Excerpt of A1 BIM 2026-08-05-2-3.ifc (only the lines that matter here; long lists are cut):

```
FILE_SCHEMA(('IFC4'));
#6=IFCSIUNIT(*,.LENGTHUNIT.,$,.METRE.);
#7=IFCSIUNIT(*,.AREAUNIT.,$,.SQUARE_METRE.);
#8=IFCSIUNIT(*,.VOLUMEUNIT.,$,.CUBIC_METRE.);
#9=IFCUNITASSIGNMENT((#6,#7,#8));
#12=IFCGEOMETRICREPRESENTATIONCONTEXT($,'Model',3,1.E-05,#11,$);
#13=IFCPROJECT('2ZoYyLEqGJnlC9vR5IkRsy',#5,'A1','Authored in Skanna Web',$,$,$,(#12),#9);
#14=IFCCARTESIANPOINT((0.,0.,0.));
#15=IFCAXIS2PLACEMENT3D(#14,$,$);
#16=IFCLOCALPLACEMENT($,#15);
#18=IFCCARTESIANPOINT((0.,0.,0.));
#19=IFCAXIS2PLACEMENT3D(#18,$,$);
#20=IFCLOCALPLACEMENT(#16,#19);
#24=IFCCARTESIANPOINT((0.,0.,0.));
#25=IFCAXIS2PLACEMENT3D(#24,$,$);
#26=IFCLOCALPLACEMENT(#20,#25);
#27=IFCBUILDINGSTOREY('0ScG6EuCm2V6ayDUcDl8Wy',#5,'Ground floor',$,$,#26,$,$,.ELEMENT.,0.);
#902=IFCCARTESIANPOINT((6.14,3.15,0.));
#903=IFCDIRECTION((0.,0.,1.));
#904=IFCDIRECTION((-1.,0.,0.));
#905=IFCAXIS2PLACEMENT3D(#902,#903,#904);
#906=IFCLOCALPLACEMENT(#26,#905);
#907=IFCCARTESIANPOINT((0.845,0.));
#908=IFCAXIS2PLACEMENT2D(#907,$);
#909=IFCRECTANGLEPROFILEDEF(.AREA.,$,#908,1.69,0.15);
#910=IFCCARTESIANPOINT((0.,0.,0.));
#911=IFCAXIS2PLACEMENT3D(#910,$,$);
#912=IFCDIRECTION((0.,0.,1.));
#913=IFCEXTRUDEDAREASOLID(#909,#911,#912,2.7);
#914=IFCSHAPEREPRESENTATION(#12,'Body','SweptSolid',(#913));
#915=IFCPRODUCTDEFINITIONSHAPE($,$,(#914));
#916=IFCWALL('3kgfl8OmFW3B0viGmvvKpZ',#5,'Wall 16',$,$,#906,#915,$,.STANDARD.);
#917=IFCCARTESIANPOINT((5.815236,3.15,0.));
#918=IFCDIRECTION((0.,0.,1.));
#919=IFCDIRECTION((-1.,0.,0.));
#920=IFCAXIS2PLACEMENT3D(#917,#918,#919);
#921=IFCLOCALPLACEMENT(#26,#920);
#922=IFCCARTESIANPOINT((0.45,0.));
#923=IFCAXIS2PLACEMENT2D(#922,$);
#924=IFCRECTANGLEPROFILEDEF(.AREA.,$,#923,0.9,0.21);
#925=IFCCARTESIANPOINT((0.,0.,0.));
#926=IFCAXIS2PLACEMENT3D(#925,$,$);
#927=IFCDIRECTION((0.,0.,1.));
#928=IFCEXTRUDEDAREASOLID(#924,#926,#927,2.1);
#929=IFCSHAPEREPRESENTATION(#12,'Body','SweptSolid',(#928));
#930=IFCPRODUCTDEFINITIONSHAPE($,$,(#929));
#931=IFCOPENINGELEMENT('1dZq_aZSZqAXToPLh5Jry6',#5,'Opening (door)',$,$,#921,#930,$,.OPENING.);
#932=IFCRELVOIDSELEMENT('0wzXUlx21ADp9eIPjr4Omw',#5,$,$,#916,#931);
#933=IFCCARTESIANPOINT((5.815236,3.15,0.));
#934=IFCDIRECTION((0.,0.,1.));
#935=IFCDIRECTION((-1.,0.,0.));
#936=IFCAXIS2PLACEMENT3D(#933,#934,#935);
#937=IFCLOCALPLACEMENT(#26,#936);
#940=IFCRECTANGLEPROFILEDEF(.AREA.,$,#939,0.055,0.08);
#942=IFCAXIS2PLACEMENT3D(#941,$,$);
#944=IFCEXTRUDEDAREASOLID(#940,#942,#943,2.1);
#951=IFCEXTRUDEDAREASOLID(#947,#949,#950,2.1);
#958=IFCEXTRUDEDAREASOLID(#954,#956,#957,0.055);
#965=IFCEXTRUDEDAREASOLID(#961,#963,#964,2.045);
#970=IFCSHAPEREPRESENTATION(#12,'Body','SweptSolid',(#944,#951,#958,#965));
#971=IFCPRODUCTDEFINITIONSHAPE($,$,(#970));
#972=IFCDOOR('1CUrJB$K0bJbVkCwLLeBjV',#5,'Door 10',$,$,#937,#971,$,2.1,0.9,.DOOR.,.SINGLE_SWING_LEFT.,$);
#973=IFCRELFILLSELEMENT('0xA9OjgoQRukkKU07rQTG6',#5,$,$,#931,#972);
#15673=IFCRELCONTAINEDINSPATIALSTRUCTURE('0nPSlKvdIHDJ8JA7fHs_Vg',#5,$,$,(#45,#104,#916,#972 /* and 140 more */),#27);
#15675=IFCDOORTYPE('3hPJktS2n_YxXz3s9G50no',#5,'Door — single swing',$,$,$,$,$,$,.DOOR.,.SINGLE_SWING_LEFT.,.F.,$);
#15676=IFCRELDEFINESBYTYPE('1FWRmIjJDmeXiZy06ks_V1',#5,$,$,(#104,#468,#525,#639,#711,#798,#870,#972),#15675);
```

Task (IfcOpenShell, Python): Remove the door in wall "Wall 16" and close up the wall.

```python
import ifcopenshell
import ifcopenshell.api.feature
import ifcopenshell.api.root
import ifcopenshell.geom
import ifcopenshell.util.shape

model = ifcopenshell.open("A1 BIM 2026-08-05-2-3.ifc")
settings = ifcopenshell.geom.settings()


def volume(element):
    """Net volume in cubic metres, openings subtracted."""
    shape = ifcopenshell.geom.create_shape(settings, element)
    return ifcopenshell.util.shape.get_volume(shape.geometry)


door = model.by_id(972)
opening = door.FillsVoids[0].RelatingOpeningElement
wall = opening.VoidsElements[0].RelatingBuildingElement
before = volume(wall)

ifcopenshell.api.root.remove_product(model, product=door)
ifcopenshell.api.feature.remove_feature(model, feature=opening)

after = volume(wall)

print(f"wall volume {before:.3f} -> {after:.3f} m3")

model.write("A1 BIM 2026-08-05-2-3_v2.ifc")
```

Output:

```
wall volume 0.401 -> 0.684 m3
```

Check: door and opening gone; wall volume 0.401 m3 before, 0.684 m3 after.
